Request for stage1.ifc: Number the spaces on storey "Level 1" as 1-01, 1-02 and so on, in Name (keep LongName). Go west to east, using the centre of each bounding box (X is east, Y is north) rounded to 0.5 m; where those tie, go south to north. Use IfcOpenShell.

First a look at what the model holds.

```python
import ifcopenshell
import ifcopenshell.util.element
import ifcopenshell.util.placement

model = ifcopenshell.open("stage1.ifc")
print(model.schema)
storey = next(s for s in model.by_type("IfcBuildingStorey") if s.Name == "Level 1")
spaces = [e for e in ifcopenshell.util.element.get_decomposition(storey) if e.is_a("IfcSpace")]
for e in sorted(spaces, key=lambda e: e.id()):
    origin = ifcopenshell.util.placement.get_local_placement(e.ObjectPlacement)[:3, 3]
    print(e.id(), e.Name, e.LongName, origin.round(2) + 0.0, sep=" | ")
```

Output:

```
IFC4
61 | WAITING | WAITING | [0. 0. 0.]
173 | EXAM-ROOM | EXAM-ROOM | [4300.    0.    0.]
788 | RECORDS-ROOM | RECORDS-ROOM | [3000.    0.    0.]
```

```python
import ifcopenshell
import ifcopenshell.geom
import ifcopenshell.util.element
import ifcopenshell.util.shape

model = ifcopenshell.open("stage1.ifc")
settings = ifcopenshell.geom.settings()
settings.set("use-world-coords", True)


def centre(element):
    shape = ifcopenshell.geom.create_shape(settings, element)
    return ifcopenshell.util.shape.get_bbox_centroid(shape.geometry)


storey = next(s for s in model.by_type("IfcBuildingStorey") if s.Name == "Level 1")
spaces = [e for e in ifcopenshell.util.element.get_decomposition(storey) if e.is_a("IfcSpace")]

# Insertion points can sit at a corner or the storey origin, so sort by the geometry (in metres).
centres = {e: centre(e) for e in spaces}
spaces.sort(key=lambda e: (round(centres[e][0] / 0.5), centres[e][1]))

for i, e in enumerate(spaces, start=1):
    number = f"1-{i:02d}"
    e.Name = number
    print(e.id(), number)

model.write("stage1_v2.ifc")
```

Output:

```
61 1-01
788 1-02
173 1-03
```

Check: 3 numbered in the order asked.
